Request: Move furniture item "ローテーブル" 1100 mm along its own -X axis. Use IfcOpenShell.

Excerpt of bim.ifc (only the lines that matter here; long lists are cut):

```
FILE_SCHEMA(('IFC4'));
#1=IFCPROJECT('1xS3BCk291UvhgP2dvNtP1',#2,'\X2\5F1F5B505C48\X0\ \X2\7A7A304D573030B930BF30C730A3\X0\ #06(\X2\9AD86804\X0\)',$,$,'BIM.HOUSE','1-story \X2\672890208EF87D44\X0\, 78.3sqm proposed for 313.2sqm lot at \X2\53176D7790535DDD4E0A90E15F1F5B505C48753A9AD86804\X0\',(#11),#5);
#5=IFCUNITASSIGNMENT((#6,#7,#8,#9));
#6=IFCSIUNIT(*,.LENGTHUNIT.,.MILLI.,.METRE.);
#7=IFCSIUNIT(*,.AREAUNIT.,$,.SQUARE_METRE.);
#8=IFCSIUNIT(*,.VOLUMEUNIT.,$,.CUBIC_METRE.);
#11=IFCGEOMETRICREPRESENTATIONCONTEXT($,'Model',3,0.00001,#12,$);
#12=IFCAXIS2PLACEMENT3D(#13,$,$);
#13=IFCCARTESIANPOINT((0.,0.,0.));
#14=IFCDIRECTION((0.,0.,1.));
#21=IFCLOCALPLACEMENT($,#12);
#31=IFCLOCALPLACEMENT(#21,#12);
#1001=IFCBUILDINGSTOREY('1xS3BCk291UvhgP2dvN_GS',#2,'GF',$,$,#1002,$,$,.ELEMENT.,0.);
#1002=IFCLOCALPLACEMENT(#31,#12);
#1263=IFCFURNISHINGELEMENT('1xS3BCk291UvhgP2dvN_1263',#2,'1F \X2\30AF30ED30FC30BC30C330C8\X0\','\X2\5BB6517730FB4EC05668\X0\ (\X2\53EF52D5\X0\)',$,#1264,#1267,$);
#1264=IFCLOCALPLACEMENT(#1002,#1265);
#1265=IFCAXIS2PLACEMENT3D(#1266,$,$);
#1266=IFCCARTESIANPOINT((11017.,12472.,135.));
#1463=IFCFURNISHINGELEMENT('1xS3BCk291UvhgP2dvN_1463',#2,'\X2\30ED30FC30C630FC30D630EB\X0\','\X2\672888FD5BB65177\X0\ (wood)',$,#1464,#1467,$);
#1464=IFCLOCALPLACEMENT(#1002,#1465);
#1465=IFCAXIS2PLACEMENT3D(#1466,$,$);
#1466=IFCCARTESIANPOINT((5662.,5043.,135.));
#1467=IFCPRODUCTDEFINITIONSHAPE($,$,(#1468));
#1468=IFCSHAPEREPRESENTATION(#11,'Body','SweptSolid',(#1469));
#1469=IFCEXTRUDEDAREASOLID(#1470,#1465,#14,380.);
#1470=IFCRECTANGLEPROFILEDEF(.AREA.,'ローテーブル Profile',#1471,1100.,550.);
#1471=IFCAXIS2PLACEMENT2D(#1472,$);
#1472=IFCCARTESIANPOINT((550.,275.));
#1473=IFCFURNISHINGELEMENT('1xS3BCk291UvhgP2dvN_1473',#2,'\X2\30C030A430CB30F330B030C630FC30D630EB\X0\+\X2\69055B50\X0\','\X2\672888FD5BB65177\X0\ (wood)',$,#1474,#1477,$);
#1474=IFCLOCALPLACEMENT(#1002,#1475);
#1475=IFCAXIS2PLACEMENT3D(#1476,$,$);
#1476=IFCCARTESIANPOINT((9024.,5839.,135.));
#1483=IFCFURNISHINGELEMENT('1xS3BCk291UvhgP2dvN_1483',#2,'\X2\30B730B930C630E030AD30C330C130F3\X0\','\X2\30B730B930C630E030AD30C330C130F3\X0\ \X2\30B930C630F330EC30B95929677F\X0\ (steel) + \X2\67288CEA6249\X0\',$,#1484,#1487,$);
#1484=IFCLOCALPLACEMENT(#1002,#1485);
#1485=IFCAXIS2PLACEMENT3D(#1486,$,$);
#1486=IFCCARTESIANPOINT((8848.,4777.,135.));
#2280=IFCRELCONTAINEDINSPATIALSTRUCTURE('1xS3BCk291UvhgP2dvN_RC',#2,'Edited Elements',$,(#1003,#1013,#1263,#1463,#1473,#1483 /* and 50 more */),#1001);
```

```python
import ifcopenshell
import ifcopenshell.api.geometry
import ifcopenshell.util.placement
import ifcopenshell.util.unit

model = ifcopenshell.open("bim.ifc")
unit_scale = ifcopenshell.util.unit.calculate_unit_scale(model)

item = model.by_guid("1xS3BCk291UvhgP2dvN_1463")
matrix = ifcopenshell.util.placement.get_local_placement(item.ObjectPlacement)
matrix[:3, 3] -= matrix[:3, 0] * 1.1 / unit_scale
ifcopenshell.api.geometry.edit_object_placement(model, product=item, matrix=matrix, is_si=False)

print(ifcopenshell.util.placement.get_local_placement(item.ObjectPlacement).round(3) + 0.0)

model.write("bim_rev.ifc")
```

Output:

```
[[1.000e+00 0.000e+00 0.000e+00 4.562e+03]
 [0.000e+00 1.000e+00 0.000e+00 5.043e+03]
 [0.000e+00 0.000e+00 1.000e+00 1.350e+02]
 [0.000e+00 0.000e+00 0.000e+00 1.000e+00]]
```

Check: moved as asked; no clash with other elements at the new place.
